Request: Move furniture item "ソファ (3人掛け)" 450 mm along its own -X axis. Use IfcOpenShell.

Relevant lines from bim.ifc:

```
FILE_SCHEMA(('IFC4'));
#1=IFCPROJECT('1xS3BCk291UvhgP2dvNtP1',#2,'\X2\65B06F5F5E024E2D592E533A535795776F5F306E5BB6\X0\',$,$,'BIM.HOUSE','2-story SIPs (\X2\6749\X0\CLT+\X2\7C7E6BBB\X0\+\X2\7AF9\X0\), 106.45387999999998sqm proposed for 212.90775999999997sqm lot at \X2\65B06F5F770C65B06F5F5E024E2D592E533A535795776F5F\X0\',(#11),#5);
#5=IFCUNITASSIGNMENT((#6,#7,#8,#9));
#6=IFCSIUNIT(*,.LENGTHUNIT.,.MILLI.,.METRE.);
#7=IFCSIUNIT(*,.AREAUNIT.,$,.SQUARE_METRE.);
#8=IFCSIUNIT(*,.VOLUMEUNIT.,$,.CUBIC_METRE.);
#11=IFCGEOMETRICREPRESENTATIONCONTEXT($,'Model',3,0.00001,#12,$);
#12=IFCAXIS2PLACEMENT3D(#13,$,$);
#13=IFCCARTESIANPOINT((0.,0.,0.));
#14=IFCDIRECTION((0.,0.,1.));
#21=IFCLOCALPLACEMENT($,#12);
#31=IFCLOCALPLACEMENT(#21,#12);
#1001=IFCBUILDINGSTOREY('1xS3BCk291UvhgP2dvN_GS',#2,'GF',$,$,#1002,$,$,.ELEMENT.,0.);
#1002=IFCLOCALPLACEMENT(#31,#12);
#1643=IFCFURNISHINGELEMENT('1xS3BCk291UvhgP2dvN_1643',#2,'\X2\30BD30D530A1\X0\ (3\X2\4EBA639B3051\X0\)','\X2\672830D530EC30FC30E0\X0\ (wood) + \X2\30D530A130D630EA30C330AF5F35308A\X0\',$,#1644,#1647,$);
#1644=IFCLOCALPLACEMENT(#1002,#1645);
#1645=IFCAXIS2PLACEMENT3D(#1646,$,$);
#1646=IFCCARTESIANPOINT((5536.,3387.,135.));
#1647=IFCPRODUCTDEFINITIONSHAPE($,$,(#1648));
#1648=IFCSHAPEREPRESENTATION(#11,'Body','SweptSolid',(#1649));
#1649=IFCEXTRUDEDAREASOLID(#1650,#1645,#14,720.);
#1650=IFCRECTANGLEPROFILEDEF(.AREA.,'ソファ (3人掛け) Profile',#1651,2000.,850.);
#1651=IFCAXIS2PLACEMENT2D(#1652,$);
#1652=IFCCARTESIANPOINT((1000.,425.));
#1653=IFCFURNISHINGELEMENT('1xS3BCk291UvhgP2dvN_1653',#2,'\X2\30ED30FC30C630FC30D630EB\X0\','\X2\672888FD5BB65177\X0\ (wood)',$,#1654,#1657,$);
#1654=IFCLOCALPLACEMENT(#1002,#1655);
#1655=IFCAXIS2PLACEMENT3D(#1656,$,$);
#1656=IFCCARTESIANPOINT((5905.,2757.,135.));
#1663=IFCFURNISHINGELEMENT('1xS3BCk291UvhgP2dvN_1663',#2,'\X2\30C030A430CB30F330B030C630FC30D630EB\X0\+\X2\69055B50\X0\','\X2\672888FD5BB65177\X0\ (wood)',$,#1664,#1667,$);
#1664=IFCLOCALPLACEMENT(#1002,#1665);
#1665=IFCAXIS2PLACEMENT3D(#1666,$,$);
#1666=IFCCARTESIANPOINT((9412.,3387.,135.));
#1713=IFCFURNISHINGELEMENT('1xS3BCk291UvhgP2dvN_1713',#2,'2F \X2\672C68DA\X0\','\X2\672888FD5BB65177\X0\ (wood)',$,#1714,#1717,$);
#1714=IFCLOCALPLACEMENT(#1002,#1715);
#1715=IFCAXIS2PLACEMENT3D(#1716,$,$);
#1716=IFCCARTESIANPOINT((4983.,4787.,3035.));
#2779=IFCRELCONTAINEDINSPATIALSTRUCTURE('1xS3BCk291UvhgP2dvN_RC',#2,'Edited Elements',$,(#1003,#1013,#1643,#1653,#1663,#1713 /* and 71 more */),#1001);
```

```python
import ifcopenshell
import ifcopenshell.api.geometry
import ifcopenshell.util.placement

model = ifcopenshell.open("bim.ifc")

item = model.by_id(1643)
matrix = ifcopenshell.util.placement.get_local_placement(item.ObjectPlacement)
matrix[:3, 3] -= matrix[:3, 0] * 450.0
ifcopenshell.api.geometry.edit_object_placement(model, product=item, matrix=matrix, is_si=False)

print(ifcopenshell.util.placement.get_local_placement(item.ObjectPlacement).round(3) + 0.0)

model.write("bim_edited.ifc")
```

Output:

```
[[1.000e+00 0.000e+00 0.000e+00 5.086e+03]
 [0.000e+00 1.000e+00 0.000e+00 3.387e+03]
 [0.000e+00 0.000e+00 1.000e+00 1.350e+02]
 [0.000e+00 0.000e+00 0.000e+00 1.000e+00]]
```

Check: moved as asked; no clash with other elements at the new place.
